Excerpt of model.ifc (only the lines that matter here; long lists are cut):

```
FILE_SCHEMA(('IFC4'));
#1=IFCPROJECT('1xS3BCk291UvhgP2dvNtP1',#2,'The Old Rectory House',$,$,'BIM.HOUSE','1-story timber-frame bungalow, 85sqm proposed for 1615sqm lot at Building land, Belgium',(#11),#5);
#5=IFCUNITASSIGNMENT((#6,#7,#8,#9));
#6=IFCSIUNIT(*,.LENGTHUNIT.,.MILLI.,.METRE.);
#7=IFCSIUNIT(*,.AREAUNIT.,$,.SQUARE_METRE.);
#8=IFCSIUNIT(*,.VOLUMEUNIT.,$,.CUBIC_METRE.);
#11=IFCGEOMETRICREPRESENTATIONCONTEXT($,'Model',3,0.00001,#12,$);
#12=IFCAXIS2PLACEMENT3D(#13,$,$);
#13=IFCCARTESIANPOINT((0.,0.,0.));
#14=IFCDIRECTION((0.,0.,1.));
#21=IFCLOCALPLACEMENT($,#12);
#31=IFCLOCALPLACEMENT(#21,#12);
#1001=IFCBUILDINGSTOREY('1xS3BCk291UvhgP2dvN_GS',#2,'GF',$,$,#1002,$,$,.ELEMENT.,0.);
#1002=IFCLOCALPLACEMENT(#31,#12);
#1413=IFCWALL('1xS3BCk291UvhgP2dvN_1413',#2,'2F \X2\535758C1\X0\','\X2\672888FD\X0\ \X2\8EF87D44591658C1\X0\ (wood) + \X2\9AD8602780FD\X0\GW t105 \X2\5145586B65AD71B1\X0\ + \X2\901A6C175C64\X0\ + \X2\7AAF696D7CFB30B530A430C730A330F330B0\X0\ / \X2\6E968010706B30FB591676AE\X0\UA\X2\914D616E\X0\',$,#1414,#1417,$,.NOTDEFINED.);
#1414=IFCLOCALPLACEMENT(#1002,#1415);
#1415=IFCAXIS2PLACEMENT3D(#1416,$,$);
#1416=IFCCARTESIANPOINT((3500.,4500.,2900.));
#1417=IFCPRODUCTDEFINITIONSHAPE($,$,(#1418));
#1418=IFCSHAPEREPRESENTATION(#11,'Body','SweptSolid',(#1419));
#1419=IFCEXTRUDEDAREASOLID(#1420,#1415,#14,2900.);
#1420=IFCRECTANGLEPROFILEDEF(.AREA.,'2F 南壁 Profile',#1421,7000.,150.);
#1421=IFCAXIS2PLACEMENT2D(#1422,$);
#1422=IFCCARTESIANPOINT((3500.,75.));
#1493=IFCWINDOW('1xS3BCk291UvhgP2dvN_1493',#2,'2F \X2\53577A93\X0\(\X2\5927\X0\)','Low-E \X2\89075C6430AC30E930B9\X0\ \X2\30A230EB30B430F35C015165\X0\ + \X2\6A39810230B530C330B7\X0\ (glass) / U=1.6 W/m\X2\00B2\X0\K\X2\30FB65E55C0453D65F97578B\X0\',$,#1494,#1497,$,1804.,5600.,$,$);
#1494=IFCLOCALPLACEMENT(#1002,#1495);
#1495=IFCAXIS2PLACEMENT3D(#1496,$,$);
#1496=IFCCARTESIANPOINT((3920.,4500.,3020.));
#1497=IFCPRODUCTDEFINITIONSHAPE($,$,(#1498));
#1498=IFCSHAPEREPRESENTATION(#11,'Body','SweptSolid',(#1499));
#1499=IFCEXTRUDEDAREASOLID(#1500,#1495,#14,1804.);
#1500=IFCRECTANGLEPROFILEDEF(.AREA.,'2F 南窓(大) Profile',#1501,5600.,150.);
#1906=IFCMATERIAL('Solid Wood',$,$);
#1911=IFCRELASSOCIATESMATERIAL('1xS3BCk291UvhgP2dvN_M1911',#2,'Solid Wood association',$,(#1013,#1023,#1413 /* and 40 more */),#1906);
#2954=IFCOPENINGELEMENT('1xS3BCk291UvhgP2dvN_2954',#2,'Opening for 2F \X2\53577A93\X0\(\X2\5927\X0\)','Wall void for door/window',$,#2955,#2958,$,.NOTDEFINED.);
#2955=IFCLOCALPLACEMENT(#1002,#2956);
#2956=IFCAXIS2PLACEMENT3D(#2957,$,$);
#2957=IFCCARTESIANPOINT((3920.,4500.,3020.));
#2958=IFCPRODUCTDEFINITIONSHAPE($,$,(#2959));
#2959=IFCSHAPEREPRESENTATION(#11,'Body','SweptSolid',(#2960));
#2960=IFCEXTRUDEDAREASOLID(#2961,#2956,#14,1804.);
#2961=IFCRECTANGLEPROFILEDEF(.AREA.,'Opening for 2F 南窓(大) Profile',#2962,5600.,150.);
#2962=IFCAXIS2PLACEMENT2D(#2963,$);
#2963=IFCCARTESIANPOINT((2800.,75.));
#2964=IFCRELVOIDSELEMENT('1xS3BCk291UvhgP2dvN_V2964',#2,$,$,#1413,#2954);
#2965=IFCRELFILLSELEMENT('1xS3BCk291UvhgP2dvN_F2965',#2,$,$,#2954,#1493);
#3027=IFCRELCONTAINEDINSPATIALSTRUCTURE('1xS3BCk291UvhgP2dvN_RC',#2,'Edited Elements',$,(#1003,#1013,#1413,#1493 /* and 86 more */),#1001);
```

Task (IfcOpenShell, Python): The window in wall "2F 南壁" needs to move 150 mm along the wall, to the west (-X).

```python
import ifcopenshell
import ifcopenshell.api.geometry
import ifcopenshell.util.placement

model = ifcopenshell.open("model.ifc")

window = model.by_id(1493)
opening = window.FillsVoids[0].RelatingOpeningElement
wall = opening.VoidsElements[0].RelatingBuildingElement

wall_matrix = ifcopenshell.util.placement.get_local_placement(wall.ObjectPlacement)
shift = wall_matrix[:3, 0] * -150.0
before = ifcopenshell.util.placement.get_local_placement(window.ObjectPlacement)[:3, 3].copy()

# The window is not placed relative to its opening, so move both.
for product in (opening, window):
    matrix = ifcopenshell.util.placement.get_local_placement(product.ObjectPlacement)
    matrix[:3, 3] += shift
    ifcopenshell.api.geometry.edit_object_placement(model, product=product, matrix=matrix, is_si=False)

after = ifcopenshell.util.placement.get_local_placement(window.ObjectPlacement)[:3, 3]
print("window moved by", (after - before).round(3) + 0.0)

model.write("model-out.ifc")
```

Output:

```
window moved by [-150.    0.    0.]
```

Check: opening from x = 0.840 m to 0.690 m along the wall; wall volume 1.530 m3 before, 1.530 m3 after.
